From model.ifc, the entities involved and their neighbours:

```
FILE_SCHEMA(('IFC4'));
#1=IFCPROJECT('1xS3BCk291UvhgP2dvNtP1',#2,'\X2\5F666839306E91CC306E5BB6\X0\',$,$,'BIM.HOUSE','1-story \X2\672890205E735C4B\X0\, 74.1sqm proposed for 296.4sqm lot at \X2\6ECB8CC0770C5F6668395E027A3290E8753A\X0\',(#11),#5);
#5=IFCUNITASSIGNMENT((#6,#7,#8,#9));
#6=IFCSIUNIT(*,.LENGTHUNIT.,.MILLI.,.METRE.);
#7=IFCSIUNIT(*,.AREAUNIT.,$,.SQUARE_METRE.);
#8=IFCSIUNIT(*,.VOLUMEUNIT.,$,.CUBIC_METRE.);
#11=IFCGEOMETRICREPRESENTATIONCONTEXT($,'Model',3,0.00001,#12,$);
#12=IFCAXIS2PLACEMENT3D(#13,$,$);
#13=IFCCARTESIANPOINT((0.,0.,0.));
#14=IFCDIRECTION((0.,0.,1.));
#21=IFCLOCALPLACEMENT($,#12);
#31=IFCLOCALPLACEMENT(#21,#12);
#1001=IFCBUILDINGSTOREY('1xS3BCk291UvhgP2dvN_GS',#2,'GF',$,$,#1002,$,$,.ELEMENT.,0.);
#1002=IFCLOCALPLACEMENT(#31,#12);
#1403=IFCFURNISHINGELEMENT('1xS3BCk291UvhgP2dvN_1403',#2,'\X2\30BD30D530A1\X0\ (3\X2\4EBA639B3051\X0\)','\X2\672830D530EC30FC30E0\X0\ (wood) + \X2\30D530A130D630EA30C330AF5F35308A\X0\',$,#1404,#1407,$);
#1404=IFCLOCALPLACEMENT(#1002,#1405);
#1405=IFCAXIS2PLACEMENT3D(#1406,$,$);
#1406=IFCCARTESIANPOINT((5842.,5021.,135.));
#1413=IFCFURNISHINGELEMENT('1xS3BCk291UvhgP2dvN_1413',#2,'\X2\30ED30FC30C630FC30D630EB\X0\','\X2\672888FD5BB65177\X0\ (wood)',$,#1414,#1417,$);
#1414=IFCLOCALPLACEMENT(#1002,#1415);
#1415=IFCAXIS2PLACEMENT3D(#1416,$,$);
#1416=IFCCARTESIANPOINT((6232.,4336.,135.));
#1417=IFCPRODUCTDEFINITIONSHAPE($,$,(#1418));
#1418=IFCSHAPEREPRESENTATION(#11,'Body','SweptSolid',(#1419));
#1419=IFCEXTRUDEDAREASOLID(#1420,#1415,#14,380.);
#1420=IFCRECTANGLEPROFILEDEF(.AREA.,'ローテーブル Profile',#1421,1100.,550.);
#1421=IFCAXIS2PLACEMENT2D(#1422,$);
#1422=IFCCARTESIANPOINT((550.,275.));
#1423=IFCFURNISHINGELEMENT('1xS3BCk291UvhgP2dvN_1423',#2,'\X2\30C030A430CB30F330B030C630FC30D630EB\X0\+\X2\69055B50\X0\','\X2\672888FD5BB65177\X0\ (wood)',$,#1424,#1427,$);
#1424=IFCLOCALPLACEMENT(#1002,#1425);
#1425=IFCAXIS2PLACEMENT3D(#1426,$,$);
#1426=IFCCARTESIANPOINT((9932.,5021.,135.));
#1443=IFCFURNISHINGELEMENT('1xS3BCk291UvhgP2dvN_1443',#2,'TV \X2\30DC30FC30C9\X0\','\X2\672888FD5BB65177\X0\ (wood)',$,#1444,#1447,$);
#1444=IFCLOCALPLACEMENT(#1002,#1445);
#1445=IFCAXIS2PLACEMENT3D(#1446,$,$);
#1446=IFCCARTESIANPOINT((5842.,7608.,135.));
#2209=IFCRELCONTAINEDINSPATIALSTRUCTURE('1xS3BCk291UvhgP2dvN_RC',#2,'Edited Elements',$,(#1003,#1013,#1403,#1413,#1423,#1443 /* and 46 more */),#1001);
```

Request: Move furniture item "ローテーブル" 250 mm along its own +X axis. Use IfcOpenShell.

```python
import ifcopenshell
import ifcopenshell.api.geometry
import ifcopenshell.util.placement
import ifcopenshell.util.unit

model = ifcopenshell.open("model.ifc")
unit_scale = ifcopenshell.util.unit.calculate_unit_scale(model)

item = model.by_guid("1xS3BCk291UvhgP2dvN_1413")
matrix = ifcopenshell.util.placement.get_local_placement(item.ObjectPlacement)
matrix[:3, 3] += matrix[:3, 0] * 0.25 / unit_scale
ifcopenshell.api.geometry.edit_object_placement(model, product=item, matrix=matrix, is_si=False)

print(ifcopenshell.util.placement.get_local_placement(item.ObjectPlacement).round(3) + 0.0)

model.write("model_edited.ifc")
```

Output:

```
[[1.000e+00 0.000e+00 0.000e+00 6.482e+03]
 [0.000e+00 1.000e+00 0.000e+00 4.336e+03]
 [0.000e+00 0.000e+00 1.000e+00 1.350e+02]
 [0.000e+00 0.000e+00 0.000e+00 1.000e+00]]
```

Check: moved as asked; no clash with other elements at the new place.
